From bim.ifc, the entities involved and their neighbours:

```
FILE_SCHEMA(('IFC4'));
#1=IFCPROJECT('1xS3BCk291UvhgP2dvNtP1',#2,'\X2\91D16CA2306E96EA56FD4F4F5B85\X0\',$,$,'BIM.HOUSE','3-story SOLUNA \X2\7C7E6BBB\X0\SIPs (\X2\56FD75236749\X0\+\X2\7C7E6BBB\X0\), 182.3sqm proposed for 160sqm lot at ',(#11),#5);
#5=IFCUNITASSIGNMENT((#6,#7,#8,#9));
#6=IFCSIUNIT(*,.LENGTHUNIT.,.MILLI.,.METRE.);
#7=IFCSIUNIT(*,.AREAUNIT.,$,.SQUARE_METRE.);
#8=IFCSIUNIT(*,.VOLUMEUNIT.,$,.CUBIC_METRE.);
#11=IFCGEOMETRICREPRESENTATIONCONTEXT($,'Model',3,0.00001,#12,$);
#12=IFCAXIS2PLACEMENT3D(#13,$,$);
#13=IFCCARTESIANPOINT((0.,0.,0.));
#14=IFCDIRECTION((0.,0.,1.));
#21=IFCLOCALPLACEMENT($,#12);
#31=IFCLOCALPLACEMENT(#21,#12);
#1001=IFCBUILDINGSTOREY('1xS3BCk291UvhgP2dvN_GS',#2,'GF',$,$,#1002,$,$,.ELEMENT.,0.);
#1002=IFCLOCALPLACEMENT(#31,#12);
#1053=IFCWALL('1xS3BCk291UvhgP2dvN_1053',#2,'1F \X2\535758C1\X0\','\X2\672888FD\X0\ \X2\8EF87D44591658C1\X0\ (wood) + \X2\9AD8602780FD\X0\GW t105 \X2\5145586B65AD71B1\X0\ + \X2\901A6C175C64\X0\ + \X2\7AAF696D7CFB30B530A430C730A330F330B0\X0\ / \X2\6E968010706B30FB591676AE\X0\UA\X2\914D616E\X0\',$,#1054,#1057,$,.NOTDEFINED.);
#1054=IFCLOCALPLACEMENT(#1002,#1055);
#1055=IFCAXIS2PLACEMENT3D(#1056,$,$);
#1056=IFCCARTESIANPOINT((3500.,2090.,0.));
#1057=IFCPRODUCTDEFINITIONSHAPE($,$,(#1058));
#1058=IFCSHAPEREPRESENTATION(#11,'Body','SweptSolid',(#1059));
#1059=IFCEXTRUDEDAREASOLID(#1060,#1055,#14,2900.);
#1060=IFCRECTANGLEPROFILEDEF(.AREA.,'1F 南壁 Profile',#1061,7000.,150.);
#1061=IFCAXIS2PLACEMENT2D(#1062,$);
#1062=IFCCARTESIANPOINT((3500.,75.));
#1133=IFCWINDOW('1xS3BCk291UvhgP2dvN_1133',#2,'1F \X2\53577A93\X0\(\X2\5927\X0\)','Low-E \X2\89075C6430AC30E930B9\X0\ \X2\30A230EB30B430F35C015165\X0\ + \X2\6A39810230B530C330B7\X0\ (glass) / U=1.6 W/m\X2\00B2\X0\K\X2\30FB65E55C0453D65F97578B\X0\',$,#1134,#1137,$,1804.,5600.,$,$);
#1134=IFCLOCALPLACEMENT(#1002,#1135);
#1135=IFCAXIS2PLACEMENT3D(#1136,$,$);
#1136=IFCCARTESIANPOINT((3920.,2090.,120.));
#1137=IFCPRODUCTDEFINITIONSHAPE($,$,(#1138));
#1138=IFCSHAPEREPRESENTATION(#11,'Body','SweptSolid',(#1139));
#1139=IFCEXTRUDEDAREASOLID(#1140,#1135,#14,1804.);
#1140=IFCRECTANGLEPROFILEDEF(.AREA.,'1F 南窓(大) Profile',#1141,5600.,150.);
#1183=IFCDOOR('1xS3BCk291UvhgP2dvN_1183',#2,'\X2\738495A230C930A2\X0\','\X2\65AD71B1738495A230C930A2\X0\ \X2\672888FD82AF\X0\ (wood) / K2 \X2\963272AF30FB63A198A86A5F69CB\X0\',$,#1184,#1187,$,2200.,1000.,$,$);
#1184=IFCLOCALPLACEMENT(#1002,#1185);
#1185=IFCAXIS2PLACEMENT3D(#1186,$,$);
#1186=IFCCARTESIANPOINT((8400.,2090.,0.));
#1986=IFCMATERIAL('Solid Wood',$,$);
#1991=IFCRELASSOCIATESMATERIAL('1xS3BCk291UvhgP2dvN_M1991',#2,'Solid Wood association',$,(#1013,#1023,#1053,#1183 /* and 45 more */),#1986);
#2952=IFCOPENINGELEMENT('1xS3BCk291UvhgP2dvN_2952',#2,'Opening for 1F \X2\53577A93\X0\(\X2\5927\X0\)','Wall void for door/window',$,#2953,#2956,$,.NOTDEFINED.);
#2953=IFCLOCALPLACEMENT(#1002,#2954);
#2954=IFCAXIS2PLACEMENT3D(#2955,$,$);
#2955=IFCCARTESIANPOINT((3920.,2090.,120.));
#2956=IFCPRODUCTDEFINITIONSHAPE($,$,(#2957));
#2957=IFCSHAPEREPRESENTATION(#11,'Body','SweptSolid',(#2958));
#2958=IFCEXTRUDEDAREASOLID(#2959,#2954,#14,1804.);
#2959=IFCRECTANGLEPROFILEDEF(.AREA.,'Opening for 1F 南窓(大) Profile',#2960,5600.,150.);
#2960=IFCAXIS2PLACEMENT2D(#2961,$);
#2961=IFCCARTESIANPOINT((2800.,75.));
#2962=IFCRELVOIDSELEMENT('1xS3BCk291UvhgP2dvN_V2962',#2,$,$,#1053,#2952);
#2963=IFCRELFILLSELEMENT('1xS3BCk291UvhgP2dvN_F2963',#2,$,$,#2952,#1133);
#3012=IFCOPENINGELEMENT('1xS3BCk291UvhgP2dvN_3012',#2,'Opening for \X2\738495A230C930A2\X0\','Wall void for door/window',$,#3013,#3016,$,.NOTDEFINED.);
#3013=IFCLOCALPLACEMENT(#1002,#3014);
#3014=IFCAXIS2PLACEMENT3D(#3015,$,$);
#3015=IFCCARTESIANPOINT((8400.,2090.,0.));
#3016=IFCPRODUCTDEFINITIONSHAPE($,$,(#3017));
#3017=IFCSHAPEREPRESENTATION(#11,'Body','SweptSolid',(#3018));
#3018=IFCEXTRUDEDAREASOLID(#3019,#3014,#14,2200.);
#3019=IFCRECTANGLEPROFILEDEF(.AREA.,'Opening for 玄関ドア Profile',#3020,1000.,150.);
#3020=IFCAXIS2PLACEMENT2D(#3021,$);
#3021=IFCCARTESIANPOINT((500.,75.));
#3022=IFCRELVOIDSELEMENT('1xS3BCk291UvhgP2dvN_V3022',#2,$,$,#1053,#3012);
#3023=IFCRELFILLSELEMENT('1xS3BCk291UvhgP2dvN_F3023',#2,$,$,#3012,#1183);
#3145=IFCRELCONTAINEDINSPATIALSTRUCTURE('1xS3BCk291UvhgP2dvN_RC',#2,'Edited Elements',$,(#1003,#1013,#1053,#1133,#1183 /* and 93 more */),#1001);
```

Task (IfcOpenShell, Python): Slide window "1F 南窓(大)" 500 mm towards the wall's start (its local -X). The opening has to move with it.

```python
import ifcopenshell
import ifcopenshell.api.geometry
import ifcopenshell.util.placement
import ifcopenshell.util.unit

model = ifcopenshell.open("bim.ifc")
unit_scale = ifcopenshell.util.unit.calculate_unit_scale(model)

window = model.by_guid("1xS3BCk291UvhgP2dvN_1133")
opening = window.FillsVoids[0].RelatingOpeningElement
wall = opening.VoidsElements[0].RelatingBuildingElement

wall_matrix = ifcopenshell.util.placement.get_local_placement(wall.ObjectPlacement)
shift = wall_matrix[:3, 0] * -0.5 / unit_scale
before = ifcopenshell.util.placement.get_local_placement(window.ObjectPlacement)[:3, 3].copy()

# The window is not placed relative to its opening, so move both.
for product in (opening, window):
    matrix = ifcopenshell.util.placement.get_local_placement(product.ObjectPlacement)
    matrix[:3, 3] += shift
    ifcopenshell.api.geometry.edit_object_placement(model, product=product, matrix=matrix, is_si=False)

after = ifcopenshell.util.placement.get_local_placement(window.ObjectPlacement)[:3, 3]
print("window moved by", (after - before).round(3) + 0.0)

model.write("bim_updated.ifc")
```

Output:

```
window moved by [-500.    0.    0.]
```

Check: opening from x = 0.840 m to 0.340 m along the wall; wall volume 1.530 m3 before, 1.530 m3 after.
